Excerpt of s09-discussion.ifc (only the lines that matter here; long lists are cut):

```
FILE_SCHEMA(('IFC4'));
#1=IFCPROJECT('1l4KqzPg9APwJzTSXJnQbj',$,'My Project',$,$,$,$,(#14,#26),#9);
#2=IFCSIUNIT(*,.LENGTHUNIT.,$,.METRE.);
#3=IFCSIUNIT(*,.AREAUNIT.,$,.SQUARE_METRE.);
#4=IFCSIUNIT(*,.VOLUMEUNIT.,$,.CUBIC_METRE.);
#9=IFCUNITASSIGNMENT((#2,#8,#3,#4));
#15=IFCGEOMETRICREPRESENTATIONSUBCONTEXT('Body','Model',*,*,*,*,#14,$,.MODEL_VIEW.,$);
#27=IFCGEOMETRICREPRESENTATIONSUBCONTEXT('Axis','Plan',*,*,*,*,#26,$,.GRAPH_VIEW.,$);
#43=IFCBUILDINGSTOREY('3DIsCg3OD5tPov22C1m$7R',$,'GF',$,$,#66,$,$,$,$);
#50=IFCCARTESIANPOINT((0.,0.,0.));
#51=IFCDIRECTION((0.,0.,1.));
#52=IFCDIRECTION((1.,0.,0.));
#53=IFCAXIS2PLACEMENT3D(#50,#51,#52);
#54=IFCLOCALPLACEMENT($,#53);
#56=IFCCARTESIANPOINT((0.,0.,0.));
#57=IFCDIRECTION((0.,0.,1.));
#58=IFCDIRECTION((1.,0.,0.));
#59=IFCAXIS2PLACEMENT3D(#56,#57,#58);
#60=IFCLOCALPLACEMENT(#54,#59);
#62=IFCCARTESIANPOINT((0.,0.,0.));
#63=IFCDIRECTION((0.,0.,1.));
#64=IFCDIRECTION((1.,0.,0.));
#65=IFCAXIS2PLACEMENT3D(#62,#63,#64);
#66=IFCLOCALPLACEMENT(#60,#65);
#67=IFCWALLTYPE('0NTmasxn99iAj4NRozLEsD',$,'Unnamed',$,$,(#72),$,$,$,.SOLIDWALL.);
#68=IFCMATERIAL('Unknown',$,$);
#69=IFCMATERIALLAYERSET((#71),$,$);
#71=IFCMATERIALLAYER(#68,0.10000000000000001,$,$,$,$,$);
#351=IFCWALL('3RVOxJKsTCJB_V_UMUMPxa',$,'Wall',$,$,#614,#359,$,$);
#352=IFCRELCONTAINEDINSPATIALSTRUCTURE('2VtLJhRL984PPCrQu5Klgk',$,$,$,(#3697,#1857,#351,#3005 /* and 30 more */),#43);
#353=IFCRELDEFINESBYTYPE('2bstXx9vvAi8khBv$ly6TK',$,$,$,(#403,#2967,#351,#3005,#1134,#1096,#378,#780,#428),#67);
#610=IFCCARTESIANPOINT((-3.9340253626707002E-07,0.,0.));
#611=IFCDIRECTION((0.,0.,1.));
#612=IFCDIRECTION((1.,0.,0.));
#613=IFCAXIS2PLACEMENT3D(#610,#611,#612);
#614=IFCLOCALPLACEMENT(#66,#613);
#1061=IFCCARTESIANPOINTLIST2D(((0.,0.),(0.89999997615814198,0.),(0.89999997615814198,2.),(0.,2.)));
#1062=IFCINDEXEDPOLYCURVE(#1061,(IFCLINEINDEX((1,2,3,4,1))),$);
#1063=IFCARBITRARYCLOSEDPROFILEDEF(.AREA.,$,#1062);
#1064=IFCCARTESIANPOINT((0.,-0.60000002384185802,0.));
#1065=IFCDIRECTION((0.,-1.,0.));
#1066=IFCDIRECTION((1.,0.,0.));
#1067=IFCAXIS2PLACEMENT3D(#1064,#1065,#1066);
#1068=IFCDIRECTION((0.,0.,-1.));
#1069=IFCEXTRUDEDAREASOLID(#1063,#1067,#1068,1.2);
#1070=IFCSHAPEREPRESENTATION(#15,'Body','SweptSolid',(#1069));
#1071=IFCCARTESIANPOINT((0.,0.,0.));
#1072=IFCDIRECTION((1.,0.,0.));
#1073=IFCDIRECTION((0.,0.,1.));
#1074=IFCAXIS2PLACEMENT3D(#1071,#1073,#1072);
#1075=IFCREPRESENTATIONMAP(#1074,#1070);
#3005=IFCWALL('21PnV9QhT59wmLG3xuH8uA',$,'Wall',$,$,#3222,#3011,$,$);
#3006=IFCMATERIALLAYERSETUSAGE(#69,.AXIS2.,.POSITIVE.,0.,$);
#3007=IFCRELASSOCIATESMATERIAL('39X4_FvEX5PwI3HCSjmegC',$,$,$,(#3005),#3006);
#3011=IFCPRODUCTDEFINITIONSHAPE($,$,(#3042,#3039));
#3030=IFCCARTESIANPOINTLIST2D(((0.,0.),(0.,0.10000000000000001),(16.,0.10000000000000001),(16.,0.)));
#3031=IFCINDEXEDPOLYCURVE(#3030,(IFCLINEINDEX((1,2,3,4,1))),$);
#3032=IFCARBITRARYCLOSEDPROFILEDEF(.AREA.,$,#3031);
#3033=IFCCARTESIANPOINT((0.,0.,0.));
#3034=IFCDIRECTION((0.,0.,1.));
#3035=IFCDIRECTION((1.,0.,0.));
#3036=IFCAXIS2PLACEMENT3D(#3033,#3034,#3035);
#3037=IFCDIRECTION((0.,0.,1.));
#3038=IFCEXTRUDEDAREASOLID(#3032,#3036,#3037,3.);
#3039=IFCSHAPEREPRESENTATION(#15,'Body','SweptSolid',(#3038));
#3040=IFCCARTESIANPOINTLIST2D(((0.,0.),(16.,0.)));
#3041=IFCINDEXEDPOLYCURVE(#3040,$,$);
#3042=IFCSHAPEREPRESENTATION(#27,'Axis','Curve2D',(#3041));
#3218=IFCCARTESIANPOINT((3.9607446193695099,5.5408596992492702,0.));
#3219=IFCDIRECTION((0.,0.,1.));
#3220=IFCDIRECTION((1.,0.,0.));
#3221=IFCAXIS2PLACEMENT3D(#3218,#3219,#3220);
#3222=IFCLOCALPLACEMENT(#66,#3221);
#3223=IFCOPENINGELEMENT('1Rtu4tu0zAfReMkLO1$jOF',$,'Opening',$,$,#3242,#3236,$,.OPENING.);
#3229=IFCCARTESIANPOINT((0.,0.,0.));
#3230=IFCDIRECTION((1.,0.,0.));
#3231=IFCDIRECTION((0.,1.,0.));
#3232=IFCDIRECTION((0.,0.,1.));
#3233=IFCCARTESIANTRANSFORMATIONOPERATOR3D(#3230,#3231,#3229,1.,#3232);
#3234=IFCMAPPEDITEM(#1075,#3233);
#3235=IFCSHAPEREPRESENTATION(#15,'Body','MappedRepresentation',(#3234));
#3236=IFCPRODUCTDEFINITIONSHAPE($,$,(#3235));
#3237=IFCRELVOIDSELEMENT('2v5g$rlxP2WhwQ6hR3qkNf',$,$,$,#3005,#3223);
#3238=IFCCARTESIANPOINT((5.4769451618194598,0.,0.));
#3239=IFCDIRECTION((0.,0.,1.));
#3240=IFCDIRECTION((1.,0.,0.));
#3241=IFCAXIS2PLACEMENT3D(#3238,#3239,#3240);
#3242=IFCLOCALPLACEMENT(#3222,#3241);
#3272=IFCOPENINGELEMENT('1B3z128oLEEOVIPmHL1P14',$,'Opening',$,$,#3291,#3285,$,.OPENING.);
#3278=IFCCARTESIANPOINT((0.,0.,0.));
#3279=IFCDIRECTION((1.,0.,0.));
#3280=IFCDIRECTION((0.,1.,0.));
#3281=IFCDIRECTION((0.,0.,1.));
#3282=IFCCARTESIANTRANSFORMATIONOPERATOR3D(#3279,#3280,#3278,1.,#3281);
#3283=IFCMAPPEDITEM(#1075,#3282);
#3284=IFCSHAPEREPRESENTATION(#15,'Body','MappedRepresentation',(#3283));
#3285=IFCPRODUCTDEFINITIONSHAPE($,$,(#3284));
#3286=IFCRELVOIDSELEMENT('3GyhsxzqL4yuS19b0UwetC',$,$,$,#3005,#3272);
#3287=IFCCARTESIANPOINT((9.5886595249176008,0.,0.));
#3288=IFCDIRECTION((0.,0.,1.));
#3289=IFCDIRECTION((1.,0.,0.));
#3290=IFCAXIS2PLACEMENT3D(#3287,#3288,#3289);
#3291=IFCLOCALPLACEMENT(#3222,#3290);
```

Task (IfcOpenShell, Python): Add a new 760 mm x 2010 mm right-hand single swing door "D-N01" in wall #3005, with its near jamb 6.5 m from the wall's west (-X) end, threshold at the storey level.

```python
import numpy as np
import ifcopenshell
import ifcopenshell.api.feature
import ifcopenshell.api.geometry
import ifcopenshell.api.root
import ifcopenshell.api.spatial
import ifcopenshell.geom
import ifcopenshell.util.element
import ifcopenshell.util.placement
import ifcopenshell.util.representation
import ifcopenshell.util.shape
import ifcopenshell.util.unit

model = ifcopenshell.open("s09-discussion.ifc")
unit_scale = ifcopenshell.util.unit.calculate_unit_scale(model)
settings = ifcopenshell.geom.settings()


def volume(element):
    """Net volume in cubic metres, openings subtracted."""
    shape = ifcopenshell.geom.create_shape(settings, element)
    return ifcopenshell.util.shape.get_volume(shape.geometry)


wall = model.by_guid("21PnV9QhT59wmLG3xuH8uA")
storey = ifcopenshell.util.element.get_container(wall, ifc_class="IfcBuildingStorey")
context = ifcopenshell.util.representation.get_context(model, "Model", "Body", "MODEL_VIEW")
before = volume(wall)

width, height, from_end, sill = 0.76, 2.01, 6.5, 0.0  # metres

# The wall runs along its own X axis, and the end named is its -X end.
wall_shape = ifcopenshell.geom.create_shape(settings, wall)
x, y, z = ifcopenshell.util.shape.get_vertices(wall_shape.geometry).T
start = x.min() + from_end
face, thickness = float(y.min()), float(y.max() - y.min())
wall_matrix = ifcopenshell.util.placement.get_local_placement(wall.ObjectPlacement)
level = ifcopenshell.util.placement.get_local_placement(storey.ObjectPlacement)[2, 3]


def in_wall(x, y):
    """Placement at x, y metres in the wall's axes, at sill height."""
    matrix = wall_matrix.copy()
    matrix[:, 3] = wall_matrix @ np.array([x / unit_scale, y / unit_scale, 0.0, 1.0])
    matrix[2, 3] = level + sill / unit_scale
    return matrix


# Opening: a box that overshoots both wall faces by 50 mm.
opening = ifcopenshell.api.root.create_entity(model, ifc_class="IfcOpeningElement", predefined_type="OPENING")
box = ifcopenshell.api.geometry.add_wall_representation(
    model, context=context, length=width, height=height, thickness=thickness + 0.1
)
ifcopenshell.api.geometry.assign_representation(model, product=opening, representation=box)
ifcopenshell.api.geometry.edit_object_placement(model, product=opening, matrix=in_wall(start, face - 0.05), is_si=False)
ifcopenshell.api.feature.add_feature(model, feature=opening, element=wall)

door = ifcopenshell.api.root.create_entity(model, ifc_class="IfcDoor", name="D-N01", predefined_type="DOOR")
door.OverallWidth, door.OverallHeight = width / unit_scale, height / unit_scale
door.OperationType = "SINGLE_SWING_RIGHT"
body = ifcopenshell.api.geometry.add_door_representation(
    model,
    context=context,
    overall_width=door.OverallWidth,
    overall_height=door.OverallHeight,
    operation_type="SINGLE_SWING_RIGHT",
    lining_properties={"LiningDepth": thickness / unit_scale, "ThresholdDepth": thickness / unit_scale},
)
ifcopenshell.api.geometry.assign_representation(model, product=door, representation=body)
ifcopenshell.api.spatial.assign_container(model, products=[door], relating_structure=storey)
ifcopenshell.api.feature.add_filling(model, opening=opening, element=door)

# The lining spans the wall, so the door starts at the wall face.
ifcopenshell.api.geometry.edit_object_placement(model, product=door, matrix=in_wall(start, face), is_si=False)

after = volume(wall)

print(f"wall volume {before:.3f} -> {after:.3f} m3")

model.write("s09-discussion_updated.ifc")
```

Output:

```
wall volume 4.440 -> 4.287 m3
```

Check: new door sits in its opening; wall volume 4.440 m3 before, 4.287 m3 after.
